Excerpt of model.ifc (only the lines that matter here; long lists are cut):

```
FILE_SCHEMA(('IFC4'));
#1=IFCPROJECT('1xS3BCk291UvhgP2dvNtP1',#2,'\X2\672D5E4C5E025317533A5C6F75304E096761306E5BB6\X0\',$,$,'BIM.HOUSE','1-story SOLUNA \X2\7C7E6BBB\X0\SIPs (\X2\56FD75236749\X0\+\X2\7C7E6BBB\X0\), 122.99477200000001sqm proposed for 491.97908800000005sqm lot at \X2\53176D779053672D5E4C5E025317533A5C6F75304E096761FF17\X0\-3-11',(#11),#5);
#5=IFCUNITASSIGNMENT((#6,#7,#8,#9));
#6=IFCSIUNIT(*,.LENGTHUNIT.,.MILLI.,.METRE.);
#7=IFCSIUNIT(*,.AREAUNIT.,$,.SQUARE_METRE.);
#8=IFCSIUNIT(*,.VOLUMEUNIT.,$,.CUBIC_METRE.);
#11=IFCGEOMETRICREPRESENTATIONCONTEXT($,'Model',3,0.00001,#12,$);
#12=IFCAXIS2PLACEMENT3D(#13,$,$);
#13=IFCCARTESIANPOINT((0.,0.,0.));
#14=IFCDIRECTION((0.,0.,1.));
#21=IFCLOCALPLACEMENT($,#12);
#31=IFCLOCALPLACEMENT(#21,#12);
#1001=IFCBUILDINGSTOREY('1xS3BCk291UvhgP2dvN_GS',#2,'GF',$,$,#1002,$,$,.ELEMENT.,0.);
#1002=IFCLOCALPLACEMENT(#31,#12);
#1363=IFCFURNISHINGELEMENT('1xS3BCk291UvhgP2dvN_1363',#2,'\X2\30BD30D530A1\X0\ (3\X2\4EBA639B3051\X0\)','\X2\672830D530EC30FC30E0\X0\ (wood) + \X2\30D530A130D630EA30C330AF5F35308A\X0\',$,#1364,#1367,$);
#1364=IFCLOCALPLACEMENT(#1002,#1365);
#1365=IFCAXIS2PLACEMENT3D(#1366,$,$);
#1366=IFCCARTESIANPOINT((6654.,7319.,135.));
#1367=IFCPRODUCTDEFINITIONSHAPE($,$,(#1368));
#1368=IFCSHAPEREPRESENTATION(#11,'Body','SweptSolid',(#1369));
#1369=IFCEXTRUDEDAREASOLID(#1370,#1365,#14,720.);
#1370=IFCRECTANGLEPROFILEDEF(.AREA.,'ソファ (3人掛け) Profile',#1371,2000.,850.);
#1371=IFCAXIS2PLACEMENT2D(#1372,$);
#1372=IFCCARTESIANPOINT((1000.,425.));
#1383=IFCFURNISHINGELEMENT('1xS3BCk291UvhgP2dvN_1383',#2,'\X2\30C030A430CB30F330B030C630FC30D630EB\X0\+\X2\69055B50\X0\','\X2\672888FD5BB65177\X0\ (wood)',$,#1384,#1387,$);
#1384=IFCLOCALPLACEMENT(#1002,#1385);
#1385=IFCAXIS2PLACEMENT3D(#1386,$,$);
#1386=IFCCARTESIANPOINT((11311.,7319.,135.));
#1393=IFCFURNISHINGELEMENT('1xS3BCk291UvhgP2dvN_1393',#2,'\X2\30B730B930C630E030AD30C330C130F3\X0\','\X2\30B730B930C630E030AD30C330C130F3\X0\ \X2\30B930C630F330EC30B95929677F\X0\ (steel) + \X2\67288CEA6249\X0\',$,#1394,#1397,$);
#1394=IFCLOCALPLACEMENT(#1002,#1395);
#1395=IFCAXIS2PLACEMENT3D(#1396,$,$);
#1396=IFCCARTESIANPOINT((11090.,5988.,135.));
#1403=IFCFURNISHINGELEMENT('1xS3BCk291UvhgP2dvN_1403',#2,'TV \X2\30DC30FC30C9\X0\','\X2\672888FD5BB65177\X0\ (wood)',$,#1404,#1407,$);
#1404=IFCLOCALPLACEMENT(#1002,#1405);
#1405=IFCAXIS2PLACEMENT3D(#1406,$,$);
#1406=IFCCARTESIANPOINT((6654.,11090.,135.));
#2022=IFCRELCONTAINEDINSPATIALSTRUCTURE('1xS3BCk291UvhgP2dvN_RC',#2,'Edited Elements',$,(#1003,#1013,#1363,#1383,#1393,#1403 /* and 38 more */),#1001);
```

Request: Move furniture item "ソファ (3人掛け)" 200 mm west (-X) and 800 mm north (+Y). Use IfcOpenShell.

```python
import ifcopenshell
import ifcopenshell.api.geometry
import ifcopenshell.util.placement

model = ifcopenshell.open("model.ifc")

item = model.by_guid("1xS3BCk291UvhgP2dvN_1363")
matrix = ifcopenshell.util.placement.get_local_placement(item.ObjectPlacement)
matrix[0, 3] -= 200.0
matrix[1, 3] += 800.0
ifcopenshell.api.geometry.edit_object_placement(model, product=item, matrix=matrix, is_si=False)

print(ifcopenshell.util.placement.get_local_placement(item.ObjectPlacement).round(3) + 0.0)

model.write("model_v2.ifc")
```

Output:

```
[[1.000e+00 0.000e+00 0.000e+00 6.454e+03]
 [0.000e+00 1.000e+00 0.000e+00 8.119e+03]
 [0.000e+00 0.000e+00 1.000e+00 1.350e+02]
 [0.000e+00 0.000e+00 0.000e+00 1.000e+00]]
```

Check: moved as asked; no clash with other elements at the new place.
